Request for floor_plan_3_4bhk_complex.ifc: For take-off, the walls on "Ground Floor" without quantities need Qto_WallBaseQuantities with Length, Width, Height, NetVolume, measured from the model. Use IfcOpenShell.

First a look at what the model holds.

```python
import ifcopenshell
import ifcopenshell.util.element
import ifcopenshell.util.unit

model = ifcopenshell.open("floor_plan_3_4bhk_complex.ifc")
print(model.schema)
for unit_type in ("LENGTHUNIT", "AREAUNIT", "VOLUMEUNIT"):
    print(unit_type, ifcopenshell.util.unit.calculate_unit_scale(model, unit_type))
storey = next(s for s in model.by_type("IfcBuildingStorey") if s.Name == "Ground Floor")
walls = [e for e in ifcopenshell.util.element.get_decomposition(storey) if e.is_a("IfcWall")]
for e in sorted(walls, key=lambda e: e.id()):
    print(e.id(), e.is_a(), e.Name, list(ifcopenshell.util.element.get_psets(e, qtos_only=True)), sep=" | ")
```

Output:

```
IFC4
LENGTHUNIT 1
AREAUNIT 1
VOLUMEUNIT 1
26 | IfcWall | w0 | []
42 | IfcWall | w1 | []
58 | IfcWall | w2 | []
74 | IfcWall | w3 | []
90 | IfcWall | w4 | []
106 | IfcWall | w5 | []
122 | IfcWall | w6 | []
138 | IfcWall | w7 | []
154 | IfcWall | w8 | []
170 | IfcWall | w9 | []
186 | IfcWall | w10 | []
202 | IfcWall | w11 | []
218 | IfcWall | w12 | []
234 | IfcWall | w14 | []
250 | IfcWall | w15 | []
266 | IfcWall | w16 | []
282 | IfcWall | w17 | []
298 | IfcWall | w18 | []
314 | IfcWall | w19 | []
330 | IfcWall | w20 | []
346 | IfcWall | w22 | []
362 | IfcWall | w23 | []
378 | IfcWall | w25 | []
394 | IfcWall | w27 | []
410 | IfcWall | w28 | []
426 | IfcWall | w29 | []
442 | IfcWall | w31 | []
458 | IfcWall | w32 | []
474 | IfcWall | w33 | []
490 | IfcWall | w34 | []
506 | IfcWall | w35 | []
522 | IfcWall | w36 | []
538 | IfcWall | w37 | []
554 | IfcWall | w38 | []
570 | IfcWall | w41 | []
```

```python
import ifcopenshell
import ifcopenshell.api.pset
import ifcopenshell.geom
import ifcopenshell.util.element
import ifcopenshell.util.shape
import ifcopenshell.util.unit

model = ifcopenshell.open("floor_plan_3_4bhk_complex.ifc")
unit_scale = ifcopenshell.util.unit.calculate_unit_scale(model)
volume_scale = ifcopenshell.util.unit.calculate_unit_scale(model, "VOLUMEUNIT")
settings = ifcopenshell.geom.settings()

storey = next(s for s in model.by_type("IfcBuildingStorey") if s.Name == "Ground Floor")
walls = [e for e in ifcopenshell.util.element.get_decomposition(storey) if e.is_a("IfcWall")]

for e in sorted(walls, key=lambda e: e.id()):
    if ifcopenshell.util.element.get_psets(e, qtos_only=True, should_inherit=False):
        continue
    # Geometry comes back in metres, in the element's own axes.
    shape = ifcopenshell.geom.create_shape(settings, e)
    values = {
        "Length": ifcopenshell.util.shape.get_x(shape.geometry) / unit_scale,
        "Width": ifcopenshell.util.shape.get_y(shape.geometry) / unit_scale,
        "Height": ifcopenshell.util.shape.get_z(shape.geometry) / unit_scale,
        "NetVolume": ifcopenshell.util.shape.get_volume(shape.geometry) / volume_scale,
    }
    qto = ifcopenshell.api.pset.add_qto(model, product=e, name="Qto_WallBaseQuantities")
    ifcopenshell.api.pset.edit_qto(model, qto=qto, properties=values)
    print(e.id(), {k: round(v, 3) for k, v in values.items()})

model.write("floor_plan_3_4bhk_complex_rev.ifc")
```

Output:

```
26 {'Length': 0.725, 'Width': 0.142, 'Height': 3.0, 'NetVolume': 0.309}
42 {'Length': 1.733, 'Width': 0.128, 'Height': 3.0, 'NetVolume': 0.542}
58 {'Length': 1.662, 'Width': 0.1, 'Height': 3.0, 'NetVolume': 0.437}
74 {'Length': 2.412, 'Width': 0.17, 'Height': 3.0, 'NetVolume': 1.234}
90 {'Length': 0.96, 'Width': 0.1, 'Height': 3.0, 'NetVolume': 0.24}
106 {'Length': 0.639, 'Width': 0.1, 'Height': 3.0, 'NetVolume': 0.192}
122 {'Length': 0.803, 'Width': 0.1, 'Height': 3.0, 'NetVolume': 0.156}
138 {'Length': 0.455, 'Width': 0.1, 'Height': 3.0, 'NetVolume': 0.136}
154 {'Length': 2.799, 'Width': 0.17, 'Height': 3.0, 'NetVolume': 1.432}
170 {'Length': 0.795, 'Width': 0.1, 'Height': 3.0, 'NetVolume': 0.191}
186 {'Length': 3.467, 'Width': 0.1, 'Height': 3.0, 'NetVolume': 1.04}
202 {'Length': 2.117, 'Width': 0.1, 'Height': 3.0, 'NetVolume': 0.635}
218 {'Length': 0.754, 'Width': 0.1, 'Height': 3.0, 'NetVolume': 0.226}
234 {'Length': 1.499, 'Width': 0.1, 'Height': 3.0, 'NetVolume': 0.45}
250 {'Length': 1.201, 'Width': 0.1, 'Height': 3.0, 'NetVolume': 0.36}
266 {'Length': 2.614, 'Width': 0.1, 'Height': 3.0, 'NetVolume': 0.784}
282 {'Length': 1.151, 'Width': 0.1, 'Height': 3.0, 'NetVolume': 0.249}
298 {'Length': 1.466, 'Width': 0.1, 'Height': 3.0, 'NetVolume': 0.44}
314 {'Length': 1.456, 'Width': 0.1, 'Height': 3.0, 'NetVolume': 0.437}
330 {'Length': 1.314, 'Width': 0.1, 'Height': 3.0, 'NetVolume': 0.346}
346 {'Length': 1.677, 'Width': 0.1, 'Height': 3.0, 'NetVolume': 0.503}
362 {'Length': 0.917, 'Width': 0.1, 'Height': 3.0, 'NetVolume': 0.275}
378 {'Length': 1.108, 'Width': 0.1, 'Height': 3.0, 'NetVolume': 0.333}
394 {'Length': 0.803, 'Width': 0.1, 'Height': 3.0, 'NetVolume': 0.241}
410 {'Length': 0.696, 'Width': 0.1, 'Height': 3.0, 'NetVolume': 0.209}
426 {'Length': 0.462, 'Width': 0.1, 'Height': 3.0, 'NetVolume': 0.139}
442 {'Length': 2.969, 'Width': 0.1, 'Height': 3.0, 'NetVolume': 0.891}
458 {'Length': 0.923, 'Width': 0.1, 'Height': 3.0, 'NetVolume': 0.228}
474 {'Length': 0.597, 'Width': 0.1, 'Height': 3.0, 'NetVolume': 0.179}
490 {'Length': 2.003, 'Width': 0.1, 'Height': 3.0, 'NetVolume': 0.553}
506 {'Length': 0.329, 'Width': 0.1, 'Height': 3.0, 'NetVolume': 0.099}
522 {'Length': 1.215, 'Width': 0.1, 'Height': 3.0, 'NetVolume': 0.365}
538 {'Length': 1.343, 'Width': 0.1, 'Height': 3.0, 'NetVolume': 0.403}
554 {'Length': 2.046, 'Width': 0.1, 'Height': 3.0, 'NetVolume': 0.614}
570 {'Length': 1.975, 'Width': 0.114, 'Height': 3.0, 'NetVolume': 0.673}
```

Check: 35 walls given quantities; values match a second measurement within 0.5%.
